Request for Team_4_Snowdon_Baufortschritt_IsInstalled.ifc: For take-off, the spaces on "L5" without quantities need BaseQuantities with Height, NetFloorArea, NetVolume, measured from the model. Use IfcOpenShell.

First a look at what the model holds.

```python
import ifcopenshell
import ifcopenshell.util.element
import ifcopenshell.util.unit

model = ifcopenshell.open("Team_4_Snowdon_Baufortschritt_IsInstalled.ifc")
print(model.schema)
for unit_type in ("LENGTHUNIT", "AREAUNIT", "VOLUMEUNIT"):
    print(unit_type, ifcopenshell.util.unit.calculate_unit_scale(model, unit_type))
storey = next(s for s in model.by_type("IfcBuildingStorey") if s.Name == "L5")
spaces = [e for e in ifcopenshell.util.element.get_decomposition(storey) if e.is_a("IfcSpace")]
for e in sorted(spaces, key=lambda e: e.id()):
    print(e.id(), e.is_a(), e.Name, list(ifcopenshell.util.element.get_psets(e, qtos_only=True)), sep=" | ")
```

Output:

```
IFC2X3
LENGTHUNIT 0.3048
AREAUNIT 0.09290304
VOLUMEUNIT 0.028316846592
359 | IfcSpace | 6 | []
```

```python
import ifcopenshell
import ifcopenshell.api.pset
import ifcopenshell.geom
import ifcopenshell.util.element
import ifcopenshell.util.shape
import ifcopenshell.util.unit

model = ifcopenshell.open("Team_4_Snowdon_Baufortschritt_IsInstalled.ifc")
unit_scale = ifcopenshell.util.unit.calculate_unit_scale(model)
area_scale = ifcopenshell.util.unit.calculate_unit_scale(model, "AREAUNIT")
volume_scale = ifcopenshell.util.unit.calculate_unit_scale(model, "VOLUMEUNIT")
settings = ifcopenshell.geom.settings()

storey = next(s for s in model.by_type("IfcBuildingStorey") if s.Name == "L5")
spaces = [e for e in ifcopenshell.util.element.get_decomposition(storey) if e.is_a("IfcSpace")]

for e in sorted(spaces, key=lambda e: e.id()):
    if ifcopenshell.util.element.get_psets(e, qtos_only=True, should_inherit=False):
        continue
    # Geometry comes back in metres, in the element's own axes.
    shape = ifcopenshell.geom.create_shape(settings, e)
    values = {
        "Height": ifcopenshell.util.shape.get_z(shape.geometry) / unit_scale,
        "NetFloorArea": ifcopenshell.util.shape.get_footprint_area(shape.geometry) / area_scale,
        "NetVolume": ifcopenshell.util.shape.get_volume(shape.geometry) / volume_scale,
    }
    qto = ifcopenshell.api.pset.add_qto(model, product=e, name="BaseQuantities")
    ifcopenshell.api.pset.edit_qto(model, qto=qto, properties=values)
    print(e.id(), {k: round(v, 3) for k, v in values.items()})

model.write("Team_4_Snowdon_Baufortschritt_IsInstalled-out.ifc")
```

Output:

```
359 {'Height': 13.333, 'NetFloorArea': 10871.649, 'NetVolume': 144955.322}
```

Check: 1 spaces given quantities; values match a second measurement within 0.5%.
